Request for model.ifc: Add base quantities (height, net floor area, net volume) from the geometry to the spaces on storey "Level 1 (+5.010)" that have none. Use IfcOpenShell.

First a look at what the model holds.

```python
import ifcopenshell
import ifcopenshell.util.element
import ifcopenshell.util.unit

model = ifcopenshell.open("model.ifc")
print(model.schema)
for unit_type in ("LENGTHUNIT", "AREAUNIT", "VOLUMEUNIT"):
    print(unit_type, ifcopenshell.util.unit.calculate_unit_scale(model, unit_type))
storey = next(s for s in model.by_type("IfcBuildingStorey") if s.Name == "Level 1 (+5.010)")
spaces = [e for e in ifcopenshell.util.element.get_decomposition(storey) if e.is_a("IfcSpace")]
for e in sorted(spaces, key=lambda e: e.id()):
    print(e.id(), e.is_a(), e.Name, list(ifcopenshell.util.element.get_psets(e, qtos_only=True)), sep=" | ")
```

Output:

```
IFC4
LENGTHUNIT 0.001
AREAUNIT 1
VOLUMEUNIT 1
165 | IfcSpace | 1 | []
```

```python
import ifcopenshell
import ifcopenshell.api.pset
import ifcopenshell.geom
import ifcopenshell.util.element
import ifcopenshell.util.shape
import ifcopenshell.util.unit

model = ifcopenshell.open("model.ifc")
unit_scale = ifcopenshell.util.unit.calculate_unit_scale(model)
area_scale = ifcopenshell.util.unit.calculate_unit_scale(model, "AREAUNIT")
volume_scale = ifcopenshell.util.unit.calculate_unit_scale(model, "VOLUMEUNIT")
settings = ifcopenshell.geom.settings()

storey = next(s for s in model.by_type("IfcBuildingStorey") if s.Name == "Level 1 (+5.010)")
spaces = [e for e in ifcopenshell.util.element.get_decomposition(storey) if e.is_a("IfcSpace")]

for e in sorted(spaces, key=lambda e: e.id()):
    if ifcopenshell.util.element.get_psets(e, qtos_only=True, should_inherit=False):
        continue
    # Geometry comes back in metres, in the element's own axes.
    shape = ifcopenshell.geom.create_shape(settings, e)
    values = {
        "Height": ifcopenshell.util.shape.get_z(shape.geometry) / unit_scale,
        "NetFloorArea": ifcopenshell.util.shape.get_footprint_area(shape.geometry) / area_scale,
        "NetVolume": ifcopenshell.util.shape.get_volume(shape.geometry) / volume_scale,
    }
    qto = ifcopenshell.api.pset.add_qto(model, product=e, name="Qto_SpaceBaseQuantities")
    ifcopenshell.api.pset.edit_qto(model, qto=qto, properties=values)
    print(e.id(), {k: round(v, 3) for k, v in values.items()})

model.write("model-out.ifc")
```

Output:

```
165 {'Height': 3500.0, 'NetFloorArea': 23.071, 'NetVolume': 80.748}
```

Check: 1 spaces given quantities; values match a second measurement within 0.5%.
